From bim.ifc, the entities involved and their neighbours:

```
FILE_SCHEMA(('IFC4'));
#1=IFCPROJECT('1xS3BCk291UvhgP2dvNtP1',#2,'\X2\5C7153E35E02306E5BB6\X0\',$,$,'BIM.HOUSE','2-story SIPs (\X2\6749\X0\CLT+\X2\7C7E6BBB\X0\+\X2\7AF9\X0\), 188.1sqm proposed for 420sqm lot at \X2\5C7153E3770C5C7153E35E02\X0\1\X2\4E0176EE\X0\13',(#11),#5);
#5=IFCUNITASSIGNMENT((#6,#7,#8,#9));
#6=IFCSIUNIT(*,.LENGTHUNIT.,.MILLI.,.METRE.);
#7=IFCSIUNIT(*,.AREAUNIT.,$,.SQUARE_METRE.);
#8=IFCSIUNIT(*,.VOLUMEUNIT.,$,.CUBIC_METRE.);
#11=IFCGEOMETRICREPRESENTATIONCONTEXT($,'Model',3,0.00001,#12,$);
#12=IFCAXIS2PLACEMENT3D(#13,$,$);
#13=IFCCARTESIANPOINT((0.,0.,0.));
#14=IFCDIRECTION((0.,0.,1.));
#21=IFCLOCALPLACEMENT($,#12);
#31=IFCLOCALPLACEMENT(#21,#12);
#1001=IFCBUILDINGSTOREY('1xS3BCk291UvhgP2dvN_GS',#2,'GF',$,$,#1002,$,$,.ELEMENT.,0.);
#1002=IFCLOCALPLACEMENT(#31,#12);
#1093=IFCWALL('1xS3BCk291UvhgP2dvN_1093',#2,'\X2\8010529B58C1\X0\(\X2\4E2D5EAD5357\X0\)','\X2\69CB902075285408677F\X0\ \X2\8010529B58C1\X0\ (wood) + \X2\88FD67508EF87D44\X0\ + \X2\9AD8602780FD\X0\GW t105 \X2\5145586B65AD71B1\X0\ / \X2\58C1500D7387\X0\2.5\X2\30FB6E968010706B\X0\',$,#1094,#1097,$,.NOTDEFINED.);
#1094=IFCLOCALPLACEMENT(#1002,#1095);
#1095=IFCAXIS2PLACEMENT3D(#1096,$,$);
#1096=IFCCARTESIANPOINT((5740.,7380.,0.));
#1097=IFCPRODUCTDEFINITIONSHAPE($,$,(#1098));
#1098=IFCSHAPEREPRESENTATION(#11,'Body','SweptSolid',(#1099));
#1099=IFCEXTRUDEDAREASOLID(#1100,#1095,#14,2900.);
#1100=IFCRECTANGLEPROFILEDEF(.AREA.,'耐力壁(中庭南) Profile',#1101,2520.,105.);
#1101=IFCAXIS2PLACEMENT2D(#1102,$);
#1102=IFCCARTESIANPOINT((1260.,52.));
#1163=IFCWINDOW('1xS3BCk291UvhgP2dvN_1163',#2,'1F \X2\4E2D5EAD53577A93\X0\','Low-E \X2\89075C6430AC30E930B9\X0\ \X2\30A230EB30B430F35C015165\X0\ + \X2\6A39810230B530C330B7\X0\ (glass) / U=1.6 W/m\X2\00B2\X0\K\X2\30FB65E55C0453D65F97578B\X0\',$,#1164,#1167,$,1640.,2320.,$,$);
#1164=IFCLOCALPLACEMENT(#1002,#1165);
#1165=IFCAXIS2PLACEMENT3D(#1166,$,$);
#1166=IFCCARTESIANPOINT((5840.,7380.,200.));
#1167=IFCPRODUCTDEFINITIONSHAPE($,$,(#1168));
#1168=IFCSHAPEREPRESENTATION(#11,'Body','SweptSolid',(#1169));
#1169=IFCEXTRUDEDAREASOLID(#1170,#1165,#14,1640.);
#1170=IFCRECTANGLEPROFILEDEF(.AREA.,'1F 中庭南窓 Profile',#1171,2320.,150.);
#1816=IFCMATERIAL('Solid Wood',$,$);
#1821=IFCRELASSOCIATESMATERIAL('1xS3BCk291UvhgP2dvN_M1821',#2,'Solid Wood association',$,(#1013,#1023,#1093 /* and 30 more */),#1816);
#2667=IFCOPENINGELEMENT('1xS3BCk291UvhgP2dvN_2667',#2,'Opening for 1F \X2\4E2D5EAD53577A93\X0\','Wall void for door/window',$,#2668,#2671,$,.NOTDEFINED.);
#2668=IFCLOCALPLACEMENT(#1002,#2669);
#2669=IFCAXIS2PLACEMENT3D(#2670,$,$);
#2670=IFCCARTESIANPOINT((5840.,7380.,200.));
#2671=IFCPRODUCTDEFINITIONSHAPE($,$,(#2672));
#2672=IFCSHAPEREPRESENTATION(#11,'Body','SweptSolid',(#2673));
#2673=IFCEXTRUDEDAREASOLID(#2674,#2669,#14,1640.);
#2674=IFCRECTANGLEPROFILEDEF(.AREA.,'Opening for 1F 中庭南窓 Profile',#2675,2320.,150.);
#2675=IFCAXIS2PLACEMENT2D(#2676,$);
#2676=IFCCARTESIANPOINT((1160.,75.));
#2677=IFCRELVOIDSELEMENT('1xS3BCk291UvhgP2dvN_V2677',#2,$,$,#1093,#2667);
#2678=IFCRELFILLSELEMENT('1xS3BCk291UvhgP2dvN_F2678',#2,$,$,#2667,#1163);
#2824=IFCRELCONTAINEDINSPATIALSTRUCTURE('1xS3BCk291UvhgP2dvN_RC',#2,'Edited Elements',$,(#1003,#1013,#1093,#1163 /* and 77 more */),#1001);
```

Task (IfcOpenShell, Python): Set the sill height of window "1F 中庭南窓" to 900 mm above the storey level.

```python
import numpy as np
import ifcopenshell
import ifcopenshell.api.geometry
import ifcopenshell.geom
import ifcopenshell.util.element
import ifcopenshell.util.placement
import ifcopenshell.util.shape
import ifcopenshell.util.unit

model = ifcopenshell.open("bim.ifc")
unit_scale = ifcopenshell.util.unit.calculate_unit_scale(model)

window = model.by_guid("1xS3BCk291UvhgP2dvN_1163")
opening = window.FillsVoids[0].RelatingOpeningElement
storey = ifcopenshell.util.element.get_container(window, ifc_class="IfcBuildingStorey")
level = ifcopenshell.util.placement.get_local_placement(storey.ObjectPlacement)[2, 3]

# The opening's origin need not be at the sill, so measure its lowest point.
shape = ifcopenshell.geom.create_shape(ifcopenshell.geom.settings(), opening)
bottom = ifcopenshell.util.shape.get_shape_bottom_elevation(shape, shape.geometry) / unit_scale
dz = level + 900.0 - bottom

shift = np.array([0.0, 0.0, dz])
# The window is not placed relative to its opening, so move both.
for product in (opening, window):
    matrix = ifcopenshell.util.placement.get_local_placement(product.ObjectPlacement)
    matrix[:3, 3] += shift
    ifcopenshell.api.geometry.edit_object_placement(model, product=product, matrix=matrix, is_si=False)

print(f"moved by {dz * unit_scale:+.3f} m")

model.write("bim-out.ifc")
```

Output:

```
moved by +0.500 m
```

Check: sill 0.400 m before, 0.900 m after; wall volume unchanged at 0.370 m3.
